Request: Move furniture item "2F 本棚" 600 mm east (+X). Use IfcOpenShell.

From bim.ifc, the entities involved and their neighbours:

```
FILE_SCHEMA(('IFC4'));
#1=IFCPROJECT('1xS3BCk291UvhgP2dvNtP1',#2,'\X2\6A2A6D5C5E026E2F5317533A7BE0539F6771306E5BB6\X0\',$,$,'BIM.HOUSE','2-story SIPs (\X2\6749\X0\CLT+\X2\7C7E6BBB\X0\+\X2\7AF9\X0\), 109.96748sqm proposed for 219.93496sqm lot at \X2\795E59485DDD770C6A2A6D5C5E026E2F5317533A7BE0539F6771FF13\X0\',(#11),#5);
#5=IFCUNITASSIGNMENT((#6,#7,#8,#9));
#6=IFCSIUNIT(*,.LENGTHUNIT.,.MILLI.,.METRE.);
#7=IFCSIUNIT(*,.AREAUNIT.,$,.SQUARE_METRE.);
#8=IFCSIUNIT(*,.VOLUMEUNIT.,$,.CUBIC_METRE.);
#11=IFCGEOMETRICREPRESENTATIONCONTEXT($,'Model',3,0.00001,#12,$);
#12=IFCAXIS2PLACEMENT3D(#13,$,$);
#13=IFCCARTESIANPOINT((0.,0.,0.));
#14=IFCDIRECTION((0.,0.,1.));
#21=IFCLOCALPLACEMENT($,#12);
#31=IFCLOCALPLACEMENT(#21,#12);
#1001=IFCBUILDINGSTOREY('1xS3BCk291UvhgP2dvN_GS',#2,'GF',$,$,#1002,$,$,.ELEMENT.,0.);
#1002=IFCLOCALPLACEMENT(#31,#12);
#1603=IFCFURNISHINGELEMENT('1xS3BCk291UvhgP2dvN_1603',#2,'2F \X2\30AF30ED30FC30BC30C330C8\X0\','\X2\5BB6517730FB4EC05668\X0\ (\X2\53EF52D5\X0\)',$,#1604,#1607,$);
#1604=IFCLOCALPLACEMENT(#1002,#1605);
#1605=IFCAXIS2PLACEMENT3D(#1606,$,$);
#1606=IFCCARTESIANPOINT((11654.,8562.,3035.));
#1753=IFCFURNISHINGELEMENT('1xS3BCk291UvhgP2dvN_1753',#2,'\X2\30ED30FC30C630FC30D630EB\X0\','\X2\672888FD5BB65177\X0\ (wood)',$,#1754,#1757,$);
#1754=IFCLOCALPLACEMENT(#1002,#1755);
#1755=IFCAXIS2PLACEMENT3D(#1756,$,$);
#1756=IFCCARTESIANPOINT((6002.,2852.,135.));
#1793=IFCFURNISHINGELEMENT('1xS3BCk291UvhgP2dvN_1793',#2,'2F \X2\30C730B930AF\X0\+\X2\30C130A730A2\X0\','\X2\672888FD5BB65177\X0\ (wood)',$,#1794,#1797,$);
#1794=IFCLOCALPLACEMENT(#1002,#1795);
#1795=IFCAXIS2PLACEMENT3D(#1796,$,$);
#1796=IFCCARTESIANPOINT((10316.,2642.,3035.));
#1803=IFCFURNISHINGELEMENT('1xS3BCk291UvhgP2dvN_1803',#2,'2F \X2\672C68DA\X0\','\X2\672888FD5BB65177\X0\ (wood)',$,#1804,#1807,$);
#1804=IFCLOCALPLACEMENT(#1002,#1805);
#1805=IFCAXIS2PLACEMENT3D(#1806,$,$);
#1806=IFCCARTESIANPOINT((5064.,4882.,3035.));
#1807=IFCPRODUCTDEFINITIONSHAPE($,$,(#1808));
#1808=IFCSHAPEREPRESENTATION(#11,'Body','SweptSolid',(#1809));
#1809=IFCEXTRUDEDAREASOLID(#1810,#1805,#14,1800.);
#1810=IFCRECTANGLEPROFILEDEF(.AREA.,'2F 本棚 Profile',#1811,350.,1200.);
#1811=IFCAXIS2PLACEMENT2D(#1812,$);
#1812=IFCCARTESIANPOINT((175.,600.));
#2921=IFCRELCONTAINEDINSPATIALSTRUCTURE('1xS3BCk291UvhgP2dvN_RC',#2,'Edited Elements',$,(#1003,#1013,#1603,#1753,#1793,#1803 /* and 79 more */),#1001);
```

```python
import ifcopenshell
import ifcopenshell.api.geometry
import ifcopenshell.util.placement

model = ifcopenshell.open("bim.ifc")

item = model.by_guid("1xS3BCk291UvhgP2dvN_1803")
matrix = ifcopenshell.util.placement.get_local_placement(item.ObjectPlacement)
matrix[0, 3] += 600.0
ifcopenshell.api.geometry.edit_object_placement(model, product=item, matrix=matrix, is_si=False)

print(ifcopenshell.util.placement.get_local_placement(item.ObjectPlacement).round(3) + 0.0)

model.write("bim-out.ifc")
```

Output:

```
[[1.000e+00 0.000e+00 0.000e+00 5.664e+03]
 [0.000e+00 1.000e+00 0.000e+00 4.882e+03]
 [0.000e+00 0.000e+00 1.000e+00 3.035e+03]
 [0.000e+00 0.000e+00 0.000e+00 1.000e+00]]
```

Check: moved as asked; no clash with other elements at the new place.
